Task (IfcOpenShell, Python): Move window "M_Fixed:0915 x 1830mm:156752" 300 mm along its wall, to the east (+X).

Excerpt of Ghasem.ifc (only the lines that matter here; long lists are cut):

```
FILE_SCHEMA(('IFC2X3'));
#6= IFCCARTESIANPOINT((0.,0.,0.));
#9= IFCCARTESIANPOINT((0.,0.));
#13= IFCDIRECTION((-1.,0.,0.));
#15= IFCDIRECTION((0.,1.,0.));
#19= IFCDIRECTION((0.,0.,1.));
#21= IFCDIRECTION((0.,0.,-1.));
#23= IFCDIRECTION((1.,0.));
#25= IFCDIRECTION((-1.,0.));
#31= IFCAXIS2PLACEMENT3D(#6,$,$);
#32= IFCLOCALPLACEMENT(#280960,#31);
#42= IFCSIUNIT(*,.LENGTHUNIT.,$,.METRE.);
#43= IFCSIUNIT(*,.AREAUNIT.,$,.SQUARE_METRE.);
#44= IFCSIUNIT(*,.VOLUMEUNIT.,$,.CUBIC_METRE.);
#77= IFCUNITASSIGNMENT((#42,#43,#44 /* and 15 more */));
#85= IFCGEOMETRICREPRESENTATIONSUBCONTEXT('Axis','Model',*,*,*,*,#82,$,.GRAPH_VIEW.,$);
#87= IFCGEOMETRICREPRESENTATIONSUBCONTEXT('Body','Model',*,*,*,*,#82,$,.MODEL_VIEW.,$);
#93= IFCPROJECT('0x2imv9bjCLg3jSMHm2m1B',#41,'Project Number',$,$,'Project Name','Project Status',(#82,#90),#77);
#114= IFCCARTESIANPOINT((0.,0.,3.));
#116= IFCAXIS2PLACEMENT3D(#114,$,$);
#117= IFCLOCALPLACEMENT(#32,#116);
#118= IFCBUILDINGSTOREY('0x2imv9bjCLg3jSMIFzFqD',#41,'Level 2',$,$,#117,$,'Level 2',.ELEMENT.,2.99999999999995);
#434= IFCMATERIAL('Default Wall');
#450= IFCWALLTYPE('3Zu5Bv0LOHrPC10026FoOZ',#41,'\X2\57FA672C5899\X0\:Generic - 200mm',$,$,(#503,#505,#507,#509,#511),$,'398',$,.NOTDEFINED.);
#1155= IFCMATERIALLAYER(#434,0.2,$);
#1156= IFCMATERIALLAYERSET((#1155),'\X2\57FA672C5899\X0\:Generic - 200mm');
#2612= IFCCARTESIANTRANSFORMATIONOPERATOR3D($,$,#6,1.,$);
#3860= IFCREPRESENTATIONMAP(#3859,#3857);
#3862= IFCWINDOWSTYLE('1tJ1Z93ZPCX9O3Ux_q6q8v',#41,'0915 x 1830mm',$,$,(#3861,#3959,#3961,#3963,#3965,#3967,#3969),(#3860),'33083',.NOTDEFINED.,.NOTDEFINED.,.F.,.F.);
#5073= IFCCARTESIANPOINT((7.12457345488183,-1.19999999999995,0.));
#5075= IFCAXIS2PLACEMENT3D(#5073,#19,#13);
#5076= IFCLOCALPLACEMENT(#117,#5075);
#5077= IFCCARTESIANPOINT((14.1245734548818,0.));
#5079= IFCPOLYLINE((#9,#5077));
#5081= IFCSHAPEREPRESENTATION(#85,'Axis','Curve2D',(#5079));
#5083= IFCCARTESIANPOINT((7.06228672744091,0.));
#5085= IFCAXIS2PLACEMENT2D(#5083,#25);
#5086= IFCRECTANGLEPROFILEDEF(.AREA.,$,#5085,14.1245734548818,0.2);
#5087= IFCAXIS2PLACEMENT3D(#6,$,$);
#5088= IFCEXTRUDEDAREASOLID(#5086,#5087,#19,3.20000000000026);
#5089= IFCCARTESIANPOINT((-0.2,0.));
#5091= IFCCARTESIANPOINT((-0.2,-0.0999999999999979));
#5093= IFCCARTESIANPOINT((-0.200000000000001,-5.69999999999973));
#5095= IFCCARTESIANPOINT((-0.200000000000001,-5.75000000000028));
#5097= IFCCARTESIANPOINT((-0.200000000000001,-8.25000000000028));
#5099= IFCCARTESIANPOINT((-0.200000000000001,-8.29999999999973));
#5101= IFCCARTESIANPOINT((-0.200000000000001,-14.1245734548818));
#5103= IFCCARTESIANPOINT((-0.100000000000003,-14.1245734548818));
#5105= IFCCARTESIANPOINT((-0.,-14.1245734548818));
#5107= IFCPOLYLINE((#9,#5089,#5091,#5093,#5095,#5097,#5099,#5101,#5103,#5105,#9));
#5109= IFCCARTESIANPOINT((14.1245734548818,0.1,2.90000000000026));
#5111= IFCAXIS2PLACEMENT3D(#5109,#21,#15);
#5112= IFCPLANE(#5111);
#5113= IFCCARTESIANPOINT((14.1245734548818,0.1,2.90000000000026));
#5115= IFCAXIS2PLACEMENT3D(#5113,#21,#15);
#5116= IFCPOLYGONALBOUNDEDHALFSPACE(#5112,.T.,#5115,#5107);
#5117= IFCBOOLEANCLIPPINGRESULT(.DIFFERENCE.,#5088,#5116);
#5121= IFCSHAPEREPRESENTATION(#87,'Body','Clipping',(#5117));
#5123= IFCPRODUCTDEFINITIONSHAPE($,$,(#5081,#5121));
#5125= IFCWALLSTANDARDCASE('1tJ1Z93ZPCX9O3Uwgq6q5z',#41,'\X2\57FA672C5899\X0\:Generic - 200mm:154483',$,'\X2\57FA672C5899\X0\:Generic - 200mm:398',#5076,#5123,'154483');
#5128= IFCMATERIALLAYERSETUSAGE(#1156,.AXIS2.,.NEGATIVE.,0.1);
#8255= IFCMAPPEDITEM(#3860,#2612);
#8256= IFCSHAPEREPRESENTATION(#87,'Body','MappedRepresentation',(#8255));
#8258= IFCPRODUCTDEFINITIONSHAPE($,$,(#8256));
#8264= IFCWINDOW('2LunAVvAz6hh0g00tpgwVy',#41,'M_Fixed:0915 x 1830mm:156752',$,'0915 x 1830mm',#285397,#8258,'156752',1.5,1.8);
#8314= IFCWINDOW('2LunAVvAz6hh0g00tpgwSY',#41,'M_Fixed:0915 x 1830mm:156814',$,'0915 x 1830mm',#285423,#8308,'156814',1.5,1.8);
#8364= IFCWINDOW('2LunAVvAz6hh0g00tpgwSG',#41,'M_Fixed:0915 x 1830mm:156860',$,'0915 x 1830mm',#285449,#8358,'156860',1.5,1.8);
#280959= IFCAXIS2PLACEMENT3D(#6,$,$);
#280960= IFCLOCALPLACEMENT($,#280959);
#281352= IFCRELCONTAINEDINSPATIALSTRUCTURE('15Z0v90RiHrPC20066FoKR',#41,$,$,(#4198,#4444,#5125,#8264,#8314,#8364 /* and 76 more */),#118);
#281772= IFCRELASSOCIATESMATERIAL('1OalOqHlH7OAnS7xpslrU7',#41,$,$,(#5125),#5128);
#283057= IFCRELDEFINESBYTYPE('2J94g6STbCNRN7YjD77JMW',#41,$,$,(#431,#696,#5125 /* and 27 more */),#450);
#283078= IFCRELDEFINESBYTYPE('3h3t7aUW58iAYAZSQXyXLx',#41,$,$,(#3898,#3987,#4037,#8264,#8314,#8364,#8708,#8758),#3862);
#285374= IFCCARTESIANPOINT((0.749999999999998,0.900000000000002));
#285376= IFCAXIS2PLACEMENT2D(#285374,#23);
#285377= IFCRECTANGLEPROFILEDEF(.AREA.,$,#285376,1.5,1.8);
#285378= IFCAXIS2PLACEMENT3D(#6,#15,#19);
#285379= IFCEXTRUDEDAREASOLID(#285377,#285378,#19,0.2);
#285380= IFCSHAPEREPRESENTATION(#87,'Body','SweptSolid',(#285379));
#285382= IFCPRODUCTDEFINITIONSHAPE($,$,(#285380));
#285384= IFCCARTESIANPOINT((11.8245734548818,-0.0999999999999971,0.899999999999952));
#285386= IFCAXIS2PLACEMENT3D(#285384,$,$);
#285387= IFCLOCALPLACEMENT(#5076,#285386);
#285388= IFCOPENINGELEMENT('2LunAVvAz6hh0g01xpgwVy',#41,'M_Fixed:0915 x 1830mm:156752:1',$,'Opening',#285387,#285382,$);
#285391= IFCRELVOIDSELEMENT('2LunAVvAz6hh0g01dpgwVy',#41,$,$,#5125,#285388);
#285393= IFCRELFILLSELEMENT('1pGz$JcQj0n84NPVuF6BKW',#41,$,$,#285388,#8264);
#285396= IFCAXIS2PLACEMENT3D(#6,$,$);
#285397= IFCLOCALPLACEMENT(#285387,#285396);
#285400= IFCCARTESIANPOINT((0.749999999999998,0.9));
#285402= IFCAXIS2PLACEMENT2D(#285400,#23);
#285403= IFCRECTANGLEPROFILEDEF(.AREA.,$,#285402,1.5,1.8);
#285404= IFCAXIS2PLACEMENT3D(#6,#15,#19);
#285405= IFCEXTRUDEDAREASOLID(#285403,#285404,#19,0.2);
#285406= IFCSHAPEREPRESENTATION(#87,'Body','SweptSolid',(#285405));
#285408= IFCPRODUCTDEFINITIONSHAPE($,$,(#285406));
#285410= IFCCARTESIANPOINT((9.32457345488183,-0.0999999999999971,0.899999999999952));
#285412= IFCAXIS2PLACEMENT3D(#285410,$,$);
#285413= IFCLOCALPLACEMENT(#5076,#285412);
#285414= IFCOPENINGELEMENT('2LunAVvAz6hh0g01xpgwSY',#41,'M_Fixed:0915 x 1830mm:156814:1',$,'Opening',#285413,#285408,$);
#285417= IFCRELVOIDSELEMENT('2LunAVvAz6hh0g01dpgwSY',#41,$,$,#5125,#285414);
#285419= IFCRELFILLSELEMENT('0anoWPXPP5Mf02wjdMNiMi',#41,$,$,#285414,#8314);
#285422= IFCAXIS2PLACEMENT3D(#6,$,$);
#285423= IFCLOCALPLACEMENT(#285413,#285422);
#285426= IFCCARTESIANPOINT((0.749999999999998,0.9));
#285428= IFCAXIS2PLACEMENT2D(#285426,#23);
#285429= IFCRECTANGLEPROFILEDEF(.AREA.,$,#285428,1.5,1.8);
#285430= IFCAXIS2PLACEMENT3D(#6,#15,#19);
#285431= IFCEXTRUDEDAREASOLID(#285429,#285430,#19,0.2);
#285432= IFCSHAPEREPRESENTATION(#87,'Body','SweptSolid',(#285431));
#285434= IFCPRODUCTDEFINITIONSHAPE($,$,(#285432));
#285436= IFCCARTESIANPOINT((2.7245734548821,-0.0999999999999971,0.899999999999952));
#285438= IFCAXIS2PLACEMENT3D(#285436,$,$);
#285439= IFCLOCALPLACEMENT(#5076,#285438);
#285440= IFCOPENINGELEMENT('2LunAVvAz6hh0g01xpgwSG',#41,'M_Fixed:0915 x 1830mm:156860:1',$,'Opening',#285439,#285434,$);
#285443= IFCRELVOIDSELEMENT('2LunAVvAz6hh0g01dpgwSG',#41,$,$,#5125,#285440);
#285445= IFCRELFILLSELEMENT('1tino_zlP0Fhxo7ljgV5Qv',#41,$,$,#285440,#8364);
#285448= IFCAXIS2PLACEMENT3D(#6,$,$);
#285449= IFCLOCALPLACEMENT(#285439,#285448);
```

```python
import ifcopenshell
import ifcopenshell.api.geometry
import ifcopenshell.util.placement
import ifcopenshell.util.unit

model = ifcopenshell.open("Ghasem.ifc")
unit_scale = ifcopenshell.util.unit.calculate_unit_scale(model)

window = model.by_guid("2LunAVvAz6hh0g00tpgwVy")
opening = window.FillsVoids[0].RelatingOpeningElement
wall = opening.VoidsElements[0].RelatingBuildingElement

wall_matrix = ifcopenshell.util.placement.get_local_placement(wall.ObjectPlacement)
shift = wall_matrix[:3, 0] * -0.3 / unit_scale
before = ifcopenshell.util.placement.get_local_placement(window.ObjectPlacement)[:3, 3].copy()

# The window is placed relative to its opening, so it follows when the opening moves.
matrix = ifcopenshell.util.placement.get_local_placement(opening.ObjectPlacement)
matrix[:3, 3] += shift
ifcopenshell.api.geometry.edit_object_placement(
    model, product=opening, matrix=matrix, is_si=False, should_transform_children=True
)

after = ifcopenshell.util.placement.get_local_placement(window.ObjectPlacement)[:3, 3]
print("window moved by", (after - before).round(3) + 0.0)

model.write("Ghasem_rev.ifc")
```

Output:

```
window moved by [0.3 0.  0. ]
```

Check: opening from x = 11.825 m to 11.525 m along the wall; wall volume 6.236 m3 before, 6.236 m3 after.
